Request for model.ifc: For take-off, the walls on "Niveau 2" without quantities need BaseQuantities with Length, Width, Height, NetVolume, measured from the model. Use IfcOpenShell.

First a look at what the model holds.

```python
import ifcopenshell
import ifcopenshell.util.element
import ifcopenshell.util.unit

model = ifcopenshell.open("model.ifc")
print(model.schema)
for unit_type in ("LENGTHUNIT", "AREAUNIT", "VOLUMEUNIT"):
    print(unit_type, ifcopenshell.util.unit.calculate_unit_scale(model, unit_type))
storey = next(s for s in model.by_type("IfcBuildingStorey") if s.Name == "Niveau 2")
walls = [e for e in ifcopenshell.util.element.get_decomposition(storey) if e.is_a("IfcWall")]
for e in sorted(walls, key=lambda e: e.id()):
    print(e.id(), e.is_a(), e.Name, list(ifcopenshell.util.element.get_psets(e, qtos_only=True)), sep=" | ")
```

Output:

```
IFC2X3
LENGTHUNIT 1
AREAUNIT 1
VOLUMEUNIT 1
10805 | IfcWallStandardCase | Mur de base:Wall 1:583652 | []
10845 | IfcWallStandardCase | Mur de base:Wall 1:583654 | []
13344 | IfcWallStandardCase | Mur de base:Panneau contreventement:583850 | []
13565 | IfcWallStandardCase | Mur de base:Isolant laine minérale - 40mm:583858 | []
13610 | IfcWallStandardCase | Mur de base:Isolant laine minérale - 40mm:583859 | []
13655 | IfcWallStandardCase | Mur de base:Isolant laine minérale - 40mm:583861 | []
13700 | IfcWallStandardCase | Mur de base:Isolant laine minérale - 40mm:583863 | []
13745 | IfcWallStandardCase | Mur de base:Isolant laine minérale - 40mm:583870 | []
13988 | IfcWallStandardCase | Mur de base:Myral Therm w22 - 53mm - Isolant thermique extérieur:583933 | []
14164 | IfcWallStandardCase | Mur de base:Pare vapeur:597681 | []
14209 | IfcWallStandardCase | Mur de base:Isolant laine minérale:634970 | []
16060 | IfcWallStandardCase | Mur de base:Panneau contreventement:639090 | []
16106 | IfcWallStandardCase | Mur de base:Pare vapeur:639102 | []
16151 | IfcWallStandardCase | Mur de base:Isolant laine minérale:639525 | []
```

```python
import ifcopenshell
import ifcopenshell.api.pset
import ifcopenshell.geom
import ifcopenshell.util.element
import ifcopenshell.util.shape
import ifcopenshell.util.unit

model = ifcopenshell.open("model.ifc")
unit_scale = ifcopenshell.util.unit.calculate_unit_scale(model)
volume_scale = ifcopenshell.util.unit.calculate_unit_scale(model, "VOLUMEUNIT")
settings = ifcopenshell.geom.settings()

storey = next(s for s in model.by_type("IfcBuildingStorey") if s.Name == "Niveau 2")
walls = [e for e in ifcopenshell.util.element.get_decomposition(storey) if e.is_a("IfcWall")]

for e in sorted(walls, key=lambda e: e.id()):
    if ifcopenshell.util.element.get_psets(e, qtos_only=True, should_inherit=False):
        continue
    # Geometry comes back in metres, in the element's own axes.
    shape = ifcopenshell.geom.create_shape(settings, e)
    values = {
        "Length": ifcopenshell.util.shape.get_x(shape.geometry) / unit_scale,
        "Width": ifcopenshell.util.shape.get_y(shape.geometry) / unit_scale,
        "Height": ifcopenshell.util.shape.get_z(shape.geometry) / unit_scale,
        "NetVolume": ifcopenshell.util.shape.get_volume(shape.geometry) / volume_scale,
    }
    qto = ifcopenshell.api.pset.add_qto(model, product=e, name="BaseQuantities")
    ifcopenshell.api.pset.edit_qto(model, qto=qto, properties=values)
    print(e.id(), {k: round(v, 3) for k, v in values.items()})

model.write("model_v2.ifc")
```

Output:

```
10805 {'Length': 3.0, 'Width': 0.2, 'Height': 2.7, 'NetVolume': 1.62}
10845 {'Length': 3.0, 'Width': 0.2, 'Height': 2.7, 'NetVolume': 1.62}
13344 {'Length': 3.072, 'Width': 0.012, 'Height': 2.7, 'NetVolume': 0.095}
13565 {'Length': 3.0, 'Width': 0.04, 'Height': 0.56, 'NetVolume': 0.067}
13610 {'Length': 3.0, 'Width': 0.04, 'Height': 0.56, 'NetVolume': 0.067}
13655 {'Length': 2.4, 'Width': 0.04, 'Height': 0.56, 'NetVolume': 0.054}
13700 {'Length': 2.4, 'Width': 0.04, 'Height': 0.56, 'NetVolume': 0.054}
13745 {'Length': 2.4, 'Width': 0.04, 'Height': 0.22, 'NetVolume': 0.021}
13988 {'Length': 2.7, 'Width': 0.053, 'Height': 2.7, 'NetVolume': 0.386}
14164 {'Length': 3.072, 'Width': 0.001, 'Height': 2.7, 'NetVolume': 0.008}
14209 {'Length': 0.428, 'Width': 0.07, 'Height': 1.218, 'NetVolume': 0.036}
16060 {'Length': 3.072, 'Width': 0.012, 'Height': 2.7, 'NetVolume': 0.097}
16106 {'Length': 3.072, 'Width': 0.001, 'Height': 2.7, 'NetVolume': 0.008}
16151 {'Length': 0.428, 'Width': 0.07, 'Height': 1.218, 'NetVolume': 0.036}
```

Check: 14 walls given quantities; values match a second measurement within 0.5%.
